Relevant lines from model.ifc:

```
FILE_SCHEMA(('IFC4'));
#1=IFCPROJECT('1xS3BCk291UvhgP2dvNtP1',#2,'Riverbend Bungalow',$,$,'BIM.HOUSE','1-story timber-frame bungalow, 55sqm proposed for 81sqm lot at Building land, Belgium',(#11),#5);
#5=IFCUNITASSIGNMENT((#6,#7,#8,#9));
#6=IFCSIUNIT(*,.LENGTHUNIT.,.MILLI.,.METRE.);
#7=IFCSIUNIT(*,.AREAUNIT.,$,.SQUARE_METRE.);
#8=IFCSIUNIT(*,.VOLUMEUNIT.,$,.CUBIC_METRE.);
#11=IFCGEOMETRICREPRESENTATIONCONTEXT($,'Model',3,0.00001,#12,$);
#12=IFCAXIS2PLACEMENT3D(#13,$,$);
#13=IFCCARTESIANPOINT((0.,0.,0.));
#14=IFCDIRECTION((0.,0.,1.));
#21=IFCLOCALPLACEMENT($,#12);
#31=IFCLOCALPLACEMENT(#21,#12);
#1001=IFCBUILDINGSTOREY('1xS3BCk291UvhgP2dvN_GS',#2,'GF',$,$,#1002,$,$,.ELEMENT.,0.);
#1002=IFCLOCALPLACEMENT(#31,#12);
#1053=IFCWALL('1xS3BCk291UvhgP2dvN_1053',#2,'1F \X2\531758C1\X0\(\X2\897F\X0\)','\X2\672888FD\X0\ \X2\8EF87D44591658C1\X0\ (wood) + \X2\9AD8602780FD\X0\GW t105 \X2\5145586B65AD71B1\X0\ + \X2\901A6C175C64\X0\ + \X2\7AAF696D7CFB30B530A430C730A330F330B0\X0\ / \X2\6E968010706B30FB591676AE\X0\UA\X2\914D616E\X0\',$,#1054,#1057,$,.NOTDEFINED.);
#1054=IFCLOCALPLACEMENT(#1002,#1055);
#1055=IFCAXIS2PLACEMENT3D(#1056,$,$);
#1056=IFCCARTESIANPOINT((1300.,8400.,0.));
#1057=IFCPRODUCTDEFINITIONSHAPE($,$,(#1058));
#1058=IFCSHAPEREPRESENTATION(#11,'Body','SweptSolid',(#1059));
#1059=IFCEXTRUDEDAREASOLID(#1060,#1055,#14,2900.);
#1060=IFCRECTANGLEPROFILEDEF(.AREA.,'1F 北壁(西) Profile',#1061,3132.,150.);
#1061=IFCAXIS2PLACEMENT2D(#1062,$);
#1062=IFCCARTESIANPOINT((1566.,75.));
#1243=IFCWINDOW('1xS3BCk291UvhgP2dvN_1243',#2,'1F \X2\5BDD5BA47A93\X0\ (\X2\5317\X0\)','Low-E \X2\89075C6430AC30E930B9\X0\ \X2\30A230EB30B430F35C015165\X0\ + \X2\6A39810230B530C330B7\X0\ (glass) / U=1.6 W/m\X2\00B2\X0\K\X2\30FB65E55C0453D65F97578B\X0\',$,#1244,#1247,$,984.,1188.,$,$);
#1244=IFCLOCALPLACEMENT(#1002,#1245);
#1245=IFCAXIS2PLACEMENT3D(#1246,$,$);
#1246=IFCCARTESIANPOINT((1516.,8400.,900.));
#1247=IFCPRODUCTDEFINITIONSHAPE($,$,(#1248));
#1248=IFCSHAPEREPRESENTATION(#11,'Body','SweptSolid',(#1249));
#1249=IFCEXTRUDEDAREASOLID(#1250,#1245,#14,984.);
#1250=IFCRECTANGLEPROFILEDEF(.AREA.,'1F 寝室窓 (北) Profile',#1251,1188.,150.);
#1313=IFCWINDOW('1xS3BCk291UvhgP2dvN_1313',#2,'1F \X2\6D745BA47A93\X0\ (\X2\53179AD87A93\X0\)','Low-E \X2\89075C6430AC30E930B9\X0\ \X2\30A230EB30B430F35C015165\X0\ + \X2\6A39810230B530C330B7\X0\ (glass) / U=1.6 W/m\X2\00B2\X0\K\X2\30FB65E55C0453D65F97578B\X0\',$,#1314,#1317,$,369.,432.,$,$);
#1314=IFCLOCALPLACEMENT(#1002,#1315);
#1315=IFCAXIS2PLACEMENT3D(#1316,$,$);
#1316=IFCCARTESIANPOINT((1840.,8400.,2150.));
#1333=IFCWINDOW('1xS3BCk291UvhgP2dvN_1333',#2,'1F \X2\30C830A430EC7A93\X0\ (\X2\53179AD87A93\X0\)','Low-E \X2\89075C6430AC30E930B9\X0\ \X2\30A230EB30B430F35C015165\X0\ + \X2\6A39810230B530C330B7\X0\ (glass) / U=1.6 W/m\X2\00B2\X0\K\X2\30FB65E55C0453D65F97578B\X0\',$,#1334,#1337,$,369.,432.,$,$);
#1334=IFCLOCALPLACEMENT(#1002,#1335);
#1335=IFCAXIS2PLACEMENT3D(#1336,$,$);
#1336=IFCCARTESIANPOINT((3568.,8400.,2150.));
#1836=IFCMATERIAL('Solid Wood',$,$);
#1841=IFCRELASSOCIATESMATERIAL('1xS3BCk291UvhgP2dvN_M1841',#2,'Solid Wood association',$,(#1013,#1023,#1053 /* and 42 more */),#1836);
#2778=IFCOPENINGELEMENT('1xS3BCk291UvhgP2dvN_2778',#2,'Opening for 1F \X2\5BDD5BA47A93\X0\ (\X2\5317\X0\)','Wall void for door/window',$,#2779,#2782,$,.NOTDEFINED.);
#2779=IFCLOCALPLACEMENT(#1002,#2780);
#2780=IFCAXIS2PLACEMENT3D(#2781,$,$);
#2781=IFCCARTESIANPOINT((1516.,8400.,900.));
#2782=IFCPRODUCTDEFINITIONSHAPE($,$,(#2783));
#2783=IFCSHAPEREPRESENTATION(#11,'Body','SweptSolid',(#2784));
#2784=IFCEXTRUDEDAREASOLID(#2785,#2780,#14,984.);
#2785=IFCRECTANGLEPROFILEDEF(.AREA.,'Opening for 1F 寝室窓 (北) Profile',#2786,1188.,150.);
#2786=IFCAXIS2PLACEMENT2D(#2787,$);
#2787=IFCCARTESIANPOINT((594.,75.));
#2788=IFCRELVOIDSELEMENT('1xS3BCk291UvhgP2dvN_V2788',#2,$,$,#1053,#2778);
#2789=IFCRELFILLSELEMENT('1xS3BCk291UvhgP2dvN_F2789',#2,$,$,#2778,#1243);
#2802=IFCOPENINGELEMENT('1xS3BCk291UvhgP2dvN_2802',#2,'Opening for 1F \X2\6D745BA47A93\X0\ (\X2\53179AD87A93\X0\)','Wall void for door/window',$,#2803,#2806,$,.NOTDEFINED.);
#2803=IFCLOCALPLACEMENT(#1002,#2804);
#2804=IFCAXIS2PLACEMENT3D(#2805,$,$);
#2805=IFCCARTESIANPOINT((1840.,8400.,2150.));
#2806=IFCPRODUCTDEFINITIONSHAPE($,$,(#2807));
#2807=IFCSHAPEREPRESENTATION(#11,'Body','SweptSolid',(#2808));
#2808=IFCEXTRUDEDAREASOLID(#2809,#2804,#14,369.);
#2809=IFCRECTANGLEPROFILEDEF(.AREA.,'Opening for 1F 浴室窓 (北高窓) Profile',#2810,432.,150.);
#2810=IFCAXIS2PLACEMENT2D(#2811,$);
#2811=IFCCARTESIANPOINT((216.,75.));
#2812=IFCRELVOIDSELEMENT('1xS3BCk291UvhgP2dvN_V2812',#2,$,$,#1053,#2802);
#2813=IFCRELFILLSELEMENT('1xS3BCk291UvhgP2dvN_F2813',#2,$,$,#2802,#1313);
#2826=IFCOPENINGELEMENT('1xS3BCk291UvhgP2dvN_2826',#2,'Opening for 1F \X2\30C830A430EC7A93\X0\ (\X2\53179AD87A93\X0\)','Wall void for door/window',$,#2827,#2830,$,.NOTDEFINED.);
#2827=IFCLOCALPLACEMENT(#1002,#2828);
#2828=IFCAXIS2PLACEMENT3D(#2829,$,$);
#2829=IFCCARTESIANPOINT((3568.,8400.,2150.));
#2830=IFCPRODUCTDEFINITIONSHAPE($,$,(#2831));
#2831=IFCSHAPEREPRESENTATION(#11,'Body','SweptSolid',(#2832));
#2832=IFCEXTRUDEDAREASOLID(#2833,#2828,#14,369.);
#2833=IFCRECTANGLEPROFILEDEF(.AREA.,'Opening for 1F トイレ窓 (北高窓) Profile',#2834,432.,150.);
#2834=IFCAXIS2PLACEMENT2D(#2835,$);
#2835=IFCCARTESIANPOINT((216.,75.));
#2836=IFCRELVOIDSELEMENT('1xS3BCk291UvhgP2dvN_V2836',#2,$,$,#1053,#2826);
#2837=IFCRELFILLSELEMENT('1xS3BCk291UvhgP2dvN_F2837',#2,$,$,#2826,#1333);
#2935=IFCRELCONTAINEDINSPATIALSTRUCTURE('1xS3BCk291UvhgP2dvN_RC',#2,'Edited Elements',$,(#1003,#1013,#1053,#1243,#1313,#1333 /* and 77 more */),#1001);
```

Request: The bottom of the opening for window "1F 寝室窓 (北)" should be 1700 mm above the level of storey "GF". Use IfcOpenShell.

```python
import numpy as np
import ifcopenshell
import ifcopenshell.api.geometry
import ifcopenshell.geom
import ifcopenshell.util.element
import ifcopenshell.util.placement
import ifcopenshell.util.shape
import ifcopenshell.util.unit

model = ifcopenshell.open("model.ifc")
unit_scale = ifcopenshell.util.unit.calculate_unit_scale(model)

window = model.by_guid("1xS3BCk291UvhgP2dvN_1243")
opening = window.FillsVoids[0].RelatingOpeningElement
storey = ifcopenshell.util.element.get_container(window, ifc_class="IfcBuildingStorey")
level = ifcopenshell.util.placement.get_local_placement(storey.ObjectPlacement)[2, 3]

# The opening's origin need not be at the sill, so measure its lowest point.
shape = ifcopenshell.geom.create_shape(ifcopenshell.geom.settings(), opening)
bottom = ifcopenshell.util.shape.get_shape_bottom_elevation(shape, shape.geometry) / unit_scale
dz = level + 1.7 / unit_scale - bottom

shift = np.array([0.0, 0.0, dz])
# The window is not placed relative to its opening, so move both.
for product in (opening, window):
    matrix = ifcopenshell.util.placement.get_local_placement(product.ObjectPlacement)
    matrix[:3, 3] += shift
    ifcopenshell.api.geometry.edit_object_placement(model, product=product, matrix=matrix, is_si=False)

print(f"moved by {dz * unit_scale:+.3f} m")

model.write("model_updated.ifc")
```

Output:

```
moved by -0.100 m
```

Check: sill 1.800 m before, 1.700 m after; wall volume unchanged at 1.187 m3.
